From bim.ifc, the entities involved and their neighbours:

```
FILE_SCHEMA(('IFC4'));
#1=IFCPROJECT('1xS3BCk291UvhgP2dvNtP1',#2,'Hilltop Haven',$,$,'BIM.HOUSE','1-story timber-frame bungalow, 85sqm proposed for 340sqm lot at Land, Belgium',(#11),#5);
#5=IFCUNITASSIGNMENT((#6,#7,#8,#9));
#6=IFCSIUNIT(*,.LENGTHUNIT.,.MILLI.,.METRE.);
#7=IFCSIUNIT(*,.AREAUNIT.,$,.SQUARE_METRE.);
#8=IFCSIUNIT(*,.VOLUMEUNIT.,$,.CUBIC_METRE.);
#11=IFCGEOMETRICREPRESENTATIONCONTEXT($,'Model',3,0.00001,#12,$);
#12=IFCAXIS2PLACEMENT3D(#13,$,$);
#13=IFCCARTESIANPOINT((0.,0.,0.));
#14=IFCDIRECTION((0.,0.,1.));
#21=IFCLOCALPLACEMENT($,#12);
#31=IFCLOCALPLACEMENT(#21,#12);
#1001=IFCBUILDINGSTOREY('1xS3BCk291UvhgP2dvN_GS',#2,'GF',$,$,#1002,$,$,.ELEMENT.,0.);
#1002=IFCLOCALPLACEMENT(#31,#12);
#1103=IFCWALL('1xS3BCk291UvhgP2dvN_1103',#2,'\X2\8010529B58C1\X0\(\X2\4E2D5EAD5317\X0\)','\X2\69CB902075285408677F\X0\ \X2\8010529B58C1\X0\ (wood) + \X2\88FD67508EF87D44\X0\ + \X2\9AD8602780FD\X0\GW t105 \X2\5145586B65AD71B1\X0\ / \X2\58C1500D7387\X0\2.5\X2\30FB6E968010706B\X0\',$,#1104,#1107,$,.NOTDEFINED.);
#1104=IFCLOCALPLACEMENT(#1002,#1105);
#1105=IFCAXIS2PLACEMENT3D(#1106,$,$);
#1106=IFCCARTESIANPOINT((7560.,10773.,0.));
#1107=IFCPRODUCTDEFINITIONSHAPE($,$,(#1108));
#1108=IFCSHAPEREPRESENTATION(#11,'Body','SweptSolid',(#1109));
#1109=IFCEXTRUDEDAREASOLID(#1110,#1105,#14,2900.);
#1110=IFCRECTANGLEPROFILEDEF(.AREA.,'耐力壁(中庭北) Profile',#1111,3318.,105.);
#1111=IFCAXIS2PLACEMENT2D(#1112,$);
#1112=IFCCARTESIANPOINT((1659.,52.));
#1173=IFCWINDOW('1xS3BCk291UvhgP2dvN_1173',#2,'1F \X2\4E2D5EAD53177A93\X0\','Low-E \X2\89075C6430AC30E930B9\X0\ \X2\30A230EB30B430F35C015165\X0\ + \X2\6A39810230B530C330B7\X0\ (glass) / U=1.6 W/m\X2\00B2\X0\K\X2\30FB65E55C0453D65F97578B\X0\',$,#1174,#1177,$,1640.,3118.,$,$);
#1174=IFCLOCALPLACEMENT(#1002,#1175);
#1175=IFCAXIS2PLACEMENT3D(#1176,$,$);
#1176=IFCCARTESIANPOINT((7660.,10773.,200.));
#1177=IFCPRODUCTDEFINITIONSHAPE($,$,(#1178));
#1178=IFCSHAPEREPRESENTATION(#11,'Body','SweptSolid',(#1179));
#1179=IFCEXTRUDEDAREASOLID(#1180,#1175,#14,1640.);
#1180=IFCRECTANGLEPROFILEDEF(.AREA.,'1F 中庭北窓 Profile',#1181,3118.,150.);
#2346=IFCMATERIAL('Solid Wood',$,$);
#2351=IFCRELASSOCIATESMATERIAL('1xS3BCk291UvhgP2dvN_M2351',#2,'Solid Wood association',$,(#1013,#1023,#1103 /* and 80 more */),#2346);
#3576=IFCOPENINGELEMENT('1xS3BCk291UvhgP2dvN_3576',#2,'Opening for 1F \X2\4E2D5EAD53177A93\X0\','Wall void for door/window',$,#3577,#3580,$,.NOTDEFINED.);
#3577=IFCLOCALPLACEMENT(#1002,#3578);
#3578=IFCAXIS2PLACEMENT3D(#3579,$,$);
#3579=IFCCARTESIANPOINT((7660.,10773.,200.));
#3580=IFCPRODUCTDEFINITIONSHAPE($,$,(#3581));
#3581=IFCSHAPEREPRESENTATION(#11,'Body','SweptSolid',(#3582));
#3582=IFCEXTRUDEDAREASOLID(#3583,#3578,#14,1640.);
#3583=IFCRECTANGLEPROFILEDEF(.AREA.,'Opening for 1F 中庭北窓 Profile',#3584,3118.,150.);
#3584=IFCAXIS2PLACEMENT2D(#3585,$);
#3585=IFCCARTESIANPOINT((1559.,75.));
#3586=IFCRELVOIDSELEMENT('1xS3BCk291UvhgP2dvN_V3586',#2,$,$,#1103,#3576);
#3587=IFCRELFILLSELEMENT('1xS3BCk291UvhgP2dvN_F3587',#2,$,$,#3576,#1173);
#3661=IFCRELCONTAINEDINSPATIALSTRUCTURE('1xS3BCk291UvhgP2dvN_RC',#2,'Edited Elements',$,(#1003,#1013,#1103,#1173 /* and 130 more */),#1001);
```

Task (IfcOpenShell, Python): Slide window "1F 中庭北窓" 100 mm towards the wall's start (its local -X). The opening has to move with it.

```python
import ifcopenshell
import ifcopenshell.api.geometry
import ifcopenshell.util.placement

model = ifcopenshell.open("bim.ifc")

window = model.by_guid("1xS3BCk291UvhgP2dvN_1173")
opening = window.FillsVoids[0].RelatingOpeningElement
wall = opening.VoidsElements[0].RelatingBuildingElement

wall_matrix = ifcopenshell.util.placement.get_local_placement(wall.ObjectPlacement)
shift = wall_matrix[:3, 0] * -100.0
before = ifcopenshell.util.placement.get_local_placement(window.ObjectPlacement)[:3, 3].copy()

# The window is not placed relative to its opening, so move both.
for product in (opening, window):
    matrix = ifcopenshell.util.placement.get_local_placement(product.ObjectPlacement)
    matrix[:3, 3] += shift
    ifcopenshell.api.geometry.edit_object_placement(model, product=product, matrix=matrix, is_si=False)

after = ifcopenshell.util.placement.get_local_placement(window.ObjectPlacement)[:3, 3]
print("window moved by", (after - before).round(3) + 0.0)

model.write("bim-out.ifc")
```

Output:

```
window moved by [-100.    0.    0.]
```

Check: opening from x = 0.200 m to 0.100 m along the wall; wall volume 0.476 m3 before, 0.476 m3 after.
